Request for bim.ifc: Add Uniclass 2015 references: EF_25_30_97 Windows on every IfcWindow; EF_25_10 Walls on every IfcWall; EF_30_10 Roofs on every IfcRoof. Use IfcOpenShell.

First a look at what the model holds.

```python
import ifcopenshell

model = ifcopenshell.open("bim.ifc")
print(model.schema)
print("classifications:", [c.Name for c in model.by_type("IfcClassification")])
for ifc_class in ("IfcDoor", "IfcRoof", "IfcStair", "IfcWall", "IfcWindow"):
    print(ifc_class, len(model.by_type(ifc_class)))
```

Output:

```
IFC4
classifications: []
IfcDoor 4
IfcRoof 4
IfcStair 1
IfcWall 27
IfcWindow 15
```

```python
import ifcopenshell
import ifcopenshell.api.classification

model = ifcopenshell.open("bim.ifc")

system = ifcopenshell.api.classification.add_classification(model, classification="Uniclass 2015")

codes = {
    "IfcWindow": ("EF_25_30_97", "Windows"),
    "IfcWall": ("EF_25_10", "Walls"),
    "IfcRoof": ("EF_30_10", "Roofs"),
}
for ifc_class, (code, name) in codes.items():
    products = model.by_type(ifc_class)
    ifcopenshell.api.classification.add_reference(
        model, products=products, classification=system, identification=code, name=name
    )
    print(code, len(products))

model.write("bim_rev.ifc")
```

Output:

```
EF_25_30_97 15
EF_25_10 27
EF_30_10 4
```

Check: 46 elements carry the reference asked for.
